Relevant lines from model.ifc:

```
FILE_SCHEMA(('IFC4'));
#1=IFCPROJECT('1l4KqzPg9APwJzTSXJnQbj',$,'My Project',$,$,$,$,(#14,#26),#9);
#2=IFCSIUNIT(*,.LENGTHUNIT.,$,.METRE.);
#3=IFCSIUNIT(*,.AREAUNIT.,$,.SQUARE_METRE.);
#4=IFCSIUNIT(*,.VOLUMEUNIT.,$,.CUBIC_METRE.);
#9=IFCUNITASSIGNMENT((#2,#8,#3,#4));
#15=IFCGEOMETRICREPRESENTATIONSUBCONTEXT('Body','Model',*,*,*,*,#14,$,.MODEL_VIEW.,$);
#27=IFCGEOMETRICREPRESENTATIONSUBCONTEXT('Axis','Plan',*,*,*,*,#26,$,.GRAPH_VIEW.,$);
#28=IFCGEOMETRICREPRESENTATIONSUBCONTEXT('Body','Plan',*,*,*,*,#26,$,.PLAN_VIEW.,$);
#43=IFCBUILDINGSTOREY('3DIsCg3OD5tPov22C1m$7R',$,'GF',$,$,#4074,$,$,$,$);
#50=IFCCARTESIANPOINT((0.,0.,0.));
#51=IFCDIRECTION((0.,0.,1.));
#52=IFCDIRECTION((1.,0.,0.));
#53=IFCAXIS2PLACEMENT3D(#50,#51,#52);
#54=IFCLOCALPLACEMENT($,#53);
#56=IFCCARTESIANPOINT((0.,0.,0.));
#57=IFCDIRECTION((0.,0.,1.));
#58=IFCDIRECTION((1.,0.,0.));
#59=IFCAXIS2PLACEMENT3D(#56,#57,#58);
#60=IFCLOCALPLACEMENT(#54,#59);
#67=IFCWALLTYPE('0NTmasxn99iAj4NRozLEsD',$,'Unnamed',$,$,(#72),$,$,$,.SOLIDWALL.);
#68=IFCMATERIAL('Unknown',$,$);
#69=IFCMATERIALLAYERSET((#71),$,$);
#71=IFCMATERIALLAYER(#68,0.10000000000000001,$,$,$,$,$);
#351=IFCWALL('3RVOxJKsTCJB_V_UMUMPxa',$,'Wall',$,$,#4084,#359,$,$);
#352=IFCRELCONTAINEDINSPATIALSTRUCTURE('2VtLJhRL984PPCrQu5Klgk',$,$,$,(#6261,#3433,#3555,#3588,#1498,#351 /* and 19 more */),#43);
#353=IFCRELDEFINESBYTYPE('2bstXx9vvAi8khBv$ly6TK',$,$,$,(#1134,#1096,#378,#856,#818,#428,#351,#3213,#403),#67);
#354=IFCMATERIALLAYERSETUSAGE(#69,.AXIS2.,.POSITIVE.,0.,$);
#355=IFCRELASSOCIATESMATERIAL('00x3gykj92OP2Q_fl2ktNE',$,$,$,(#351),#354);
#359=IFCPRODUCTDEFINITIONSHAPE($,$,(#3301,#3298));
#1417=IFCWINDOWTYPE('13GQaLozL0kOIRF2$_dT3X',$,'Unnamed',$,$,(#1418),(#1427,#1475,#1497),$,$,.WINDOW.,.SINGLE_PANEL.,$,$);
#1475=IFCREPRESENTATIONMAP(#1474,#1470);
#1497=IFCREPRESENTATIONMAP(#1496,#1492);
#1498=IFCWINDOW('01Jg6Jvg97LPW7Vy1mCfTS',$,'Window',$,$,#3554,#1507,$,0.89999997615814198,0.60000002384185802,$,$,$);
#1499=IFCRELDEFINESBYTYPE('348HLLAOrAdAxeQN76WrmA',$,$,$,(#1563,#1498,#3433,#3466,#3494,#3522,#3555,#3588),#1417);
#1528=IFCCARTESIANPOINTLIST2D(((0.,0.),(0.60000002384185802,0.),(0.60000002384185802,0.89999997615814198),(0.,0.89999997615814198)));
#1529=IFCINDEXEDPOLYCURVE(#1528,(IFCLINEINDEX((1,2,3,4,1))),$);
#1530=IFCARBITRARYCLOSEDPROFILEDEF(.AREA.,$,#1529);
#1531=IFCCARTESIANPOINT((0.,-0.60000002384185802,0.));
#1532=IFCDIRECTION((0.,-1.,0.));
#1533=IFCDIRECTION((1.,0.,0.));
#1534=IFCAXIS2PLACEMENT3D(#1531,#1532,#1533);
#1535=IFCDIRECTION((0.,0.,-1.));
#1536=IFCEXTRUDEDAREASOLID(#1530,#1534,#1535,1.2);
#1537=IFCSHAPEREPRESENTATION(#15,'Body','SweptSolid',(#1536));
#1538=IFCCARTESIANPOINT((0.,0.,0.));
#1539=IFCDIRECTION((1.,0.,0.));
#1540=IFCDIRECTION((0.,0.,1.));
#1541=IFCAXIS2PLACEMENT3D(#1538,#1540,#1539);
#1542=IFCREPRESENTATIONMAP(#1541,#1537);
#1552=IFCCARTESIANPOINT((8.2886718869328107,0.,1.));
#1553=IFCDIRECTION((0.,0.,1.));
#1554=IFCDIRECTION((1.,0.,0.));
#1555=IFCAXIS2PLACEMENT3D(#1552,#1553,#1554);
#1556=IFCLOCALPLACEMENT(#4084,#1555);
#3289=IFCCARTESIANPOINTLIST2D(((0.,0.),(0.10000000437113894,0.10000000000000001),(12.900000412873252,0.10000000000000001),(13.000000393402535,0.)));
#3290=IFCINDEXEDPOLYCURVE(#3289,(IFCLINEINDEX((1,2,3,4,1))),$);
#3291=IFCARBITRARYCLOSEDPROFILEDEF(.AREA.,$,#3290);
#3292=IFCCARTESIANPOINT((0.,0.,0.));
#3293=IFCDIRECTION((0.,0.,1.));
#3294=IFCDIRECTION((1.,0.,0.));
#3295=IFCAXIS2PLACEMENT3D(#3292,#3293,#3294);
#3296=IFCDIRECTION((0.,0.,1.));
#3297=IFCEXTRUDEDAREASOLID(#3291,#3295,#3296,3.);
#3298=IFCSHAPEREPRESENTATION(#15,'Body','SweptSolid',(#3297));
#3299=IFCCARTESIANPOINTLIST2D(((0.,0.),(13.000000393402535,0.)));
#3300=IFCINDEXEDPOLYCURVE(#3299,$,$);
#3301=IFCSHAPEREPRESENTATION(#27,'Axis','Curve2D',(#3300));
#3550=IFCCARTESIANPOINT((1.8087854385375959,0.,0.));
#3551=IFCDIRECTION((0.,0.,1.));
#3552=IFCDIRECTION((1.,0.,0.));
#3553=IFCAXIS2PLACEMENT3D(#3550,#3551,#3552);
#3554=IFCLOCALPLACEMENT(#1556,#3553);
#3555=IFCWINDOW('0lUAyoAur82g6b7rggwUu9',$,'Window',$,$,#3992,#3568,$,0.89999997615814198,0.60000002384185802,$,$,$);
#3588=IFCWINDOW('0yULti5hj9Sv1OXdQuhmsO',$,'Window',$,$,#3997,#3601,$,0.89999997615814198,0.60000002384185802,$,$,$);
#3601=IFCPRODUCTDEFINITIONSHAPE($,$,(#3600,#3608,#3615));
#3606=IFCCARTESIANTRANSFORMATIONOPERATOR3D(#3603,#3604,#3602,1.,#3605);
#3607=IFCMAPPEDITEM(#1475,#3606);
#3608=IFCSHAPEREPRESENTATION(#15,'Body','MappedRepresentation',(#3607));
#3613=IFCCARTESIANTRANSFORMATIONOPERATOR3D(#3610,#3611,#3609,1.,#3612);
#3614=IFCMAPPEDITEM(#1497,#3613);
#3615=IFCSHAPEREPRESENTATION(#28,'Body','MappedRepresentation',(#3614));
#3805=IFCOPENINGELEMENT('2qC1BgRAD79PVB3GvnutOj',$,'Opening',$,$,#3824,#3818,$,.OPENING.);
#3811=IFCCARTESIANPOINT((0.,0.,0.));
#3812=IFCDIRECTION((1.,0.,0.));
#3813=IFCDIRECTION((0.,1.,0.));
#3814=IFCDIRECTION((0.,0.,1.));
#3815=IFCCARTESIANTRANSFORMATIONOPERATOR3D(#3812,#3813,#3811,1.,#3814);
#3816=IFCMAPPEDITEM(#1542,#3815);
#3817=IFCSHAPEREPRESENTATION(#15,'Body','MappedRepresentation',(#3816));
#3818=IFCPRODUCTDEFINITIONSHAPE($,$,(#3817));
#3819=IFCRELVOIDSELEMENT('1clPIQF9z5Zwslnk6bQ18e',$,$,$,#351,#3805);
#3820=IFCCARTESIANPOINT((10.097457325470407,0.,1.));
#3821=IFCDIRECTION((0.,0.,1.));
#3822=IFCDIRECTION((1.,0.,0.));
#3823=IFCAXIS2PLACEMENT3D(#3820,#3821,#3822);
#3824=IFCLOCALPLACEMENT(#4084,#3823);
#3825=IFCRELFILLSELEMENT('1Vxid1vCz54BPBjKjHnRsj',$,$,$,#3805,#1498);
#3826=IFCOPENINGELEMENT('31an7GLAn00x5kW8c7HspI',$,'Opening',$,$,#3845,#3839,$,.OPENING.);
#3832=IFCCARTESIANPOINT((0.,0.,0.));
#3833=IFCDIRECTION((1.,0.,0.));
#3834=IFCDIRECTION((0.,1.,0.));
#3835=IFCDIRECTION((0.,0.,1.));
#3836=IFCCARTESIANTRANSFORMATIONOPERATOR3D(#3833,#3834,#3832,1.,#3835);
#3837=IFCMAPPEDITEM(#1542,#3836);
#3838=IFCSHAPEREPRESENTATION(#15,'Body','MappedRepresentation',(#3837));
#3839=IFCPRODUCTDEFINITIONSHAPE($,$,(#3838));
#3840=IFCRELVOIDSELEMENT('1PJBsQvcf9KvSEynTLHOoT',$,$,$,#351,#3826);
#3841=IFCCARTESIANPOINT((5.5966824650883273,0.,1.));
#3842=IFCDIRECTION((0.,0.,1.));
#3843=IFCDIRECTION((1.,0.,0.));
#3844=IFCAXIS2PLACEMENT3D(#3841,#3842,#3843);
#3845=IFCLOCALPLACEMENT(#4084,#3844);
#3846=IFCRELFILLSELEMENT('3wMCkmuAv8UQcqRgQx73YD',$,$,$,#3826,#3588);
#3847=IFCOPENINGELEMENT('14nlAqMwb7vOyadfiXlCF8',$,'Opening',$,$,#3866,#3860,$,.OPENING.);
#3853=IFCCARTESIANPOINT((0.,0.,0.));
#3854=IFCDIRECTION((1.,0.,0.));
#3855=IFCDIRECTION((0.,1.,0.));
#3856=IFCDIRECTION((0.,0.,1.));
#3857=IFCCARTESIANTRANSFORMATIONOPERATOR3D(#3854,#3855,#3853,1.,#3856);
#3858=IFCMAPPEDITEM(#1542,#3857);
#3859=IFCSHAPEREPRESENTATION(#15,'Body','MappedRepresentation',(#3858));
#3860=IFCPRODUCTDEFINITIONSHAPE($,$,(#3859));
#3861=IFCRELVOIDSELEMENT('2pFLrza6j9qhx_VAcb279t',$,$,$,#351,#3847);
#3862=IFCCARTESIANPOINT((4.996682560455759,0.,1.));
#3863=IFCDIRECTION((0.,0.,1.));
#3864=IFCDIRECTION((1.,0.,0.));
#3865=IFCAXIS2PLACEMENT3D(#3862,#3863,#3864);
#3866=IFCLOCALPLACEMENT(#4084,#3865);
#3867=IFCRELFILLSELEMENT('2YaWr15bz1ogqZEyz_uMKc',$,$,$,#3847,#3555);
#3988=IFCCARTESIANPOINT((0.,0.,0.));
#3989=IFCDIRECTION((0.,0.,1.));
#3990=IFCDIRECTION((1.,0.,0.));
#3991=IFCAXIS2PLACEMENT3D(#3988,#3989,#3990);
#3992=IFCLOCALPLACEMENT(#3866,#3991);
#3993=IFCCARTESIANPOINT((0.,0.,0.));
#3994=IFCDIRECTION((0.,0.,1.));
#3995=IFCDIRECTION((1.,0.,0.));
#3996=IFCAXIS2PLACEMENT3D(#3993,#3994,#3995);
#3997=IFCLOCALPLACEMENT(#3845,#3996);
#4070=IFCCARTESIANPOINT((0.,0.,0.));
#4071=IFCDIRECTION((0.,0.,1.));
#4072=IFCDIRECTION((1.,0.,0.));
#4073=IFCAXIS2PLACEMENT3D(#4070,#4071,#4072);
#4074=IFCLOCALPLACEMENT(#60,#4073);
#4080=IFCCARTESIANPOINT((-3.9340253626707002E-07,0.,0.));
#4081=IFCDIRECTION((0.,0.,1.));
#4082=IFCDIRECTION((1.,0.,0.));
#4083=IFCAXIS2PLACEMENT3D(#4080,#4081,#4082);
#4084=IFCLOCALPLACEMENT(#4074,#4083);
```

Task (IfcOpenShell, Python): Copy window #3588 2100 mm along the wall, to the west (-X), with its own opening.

```python
import ifcopenshell
import ifcopenshell.api.feature
import ifcopenshell.api.geometry
import ifcopenshell.api.root
import ifcopenshell.geom
import ifcopenshell.util.element
import ifcopenshell.util.placement
import ifcopenshell.util.shape
import ifcopenshell.util.unit

model = ifcopenshell.open("model.ifc")
unit_scale = ifcopenshell.util.unit.calculate_unit_scale(model)
settings = ifcopenshell.geom.settings()


def volume(element):
    """Net volume in cubic metres, openings subtracted."""
    shape = ifcopenshell.geom.create_shape(settings, element)
    return ifcopenshell.util.shape.get_volume(shape.geometry)


window = model.by_id(3588)
opening = window.FillsVoids[0].RelatingOpeningElement
wall = opening.VoidsElements[0].RelatingBuildingElement
before = volume(wall)
shift = ifcopenshell.util.placement.get_local_placement(wall.ObjectPlacement)[:3, 0] * -2.1 / unit_scale

# copy_class copies the void relationship, type, container and properties, but no geometry.
new_opening = ifcopenshell.api.root.copy_class(model, product=opening)
new_opening.Representation = ifcopenshell.util.element.copy_deep(
    model, opening.Representation, exclude=["IfcGeometricRepresentationContext", "IfcRepresentationMap"]
)
new_window = ifcopenshell.api.root.copy_class(model, product=window)
new_window.Representation = ifcopenshell.util.element.copy_deep(
    model, window.Representation, exclude=["IfcGeometricRepresentationContext", "IfcRepresentationMap"]
)
ifcopenshell.api.feature.add_filling(model, opening=new_opening, element=new_window)

for old, new in ((opening, new_opening), (window, new_window)):
    matrix = ifcopenshell.util.placement.get_local_placement(old.ObjectPlacement)
    matrix[:3, 3] += shift
    ifcopenshell.api.geometry.edit_object_placement(model, product=new, matrix=matrix, is_si=False)

after = volume(wall)

print(f"wall volume {before:.3f} -> {after:.3f} m3")

model.write("model_rev.ifc")
```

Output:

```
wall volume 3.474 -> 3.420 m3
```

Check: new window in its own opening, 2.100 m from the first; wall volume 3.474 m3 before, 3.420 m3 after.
